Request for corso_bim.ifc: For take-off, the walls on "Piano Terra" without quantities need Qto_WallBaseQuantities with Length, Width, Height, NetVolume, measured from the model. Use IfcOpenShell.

First a look at what the model holds.

```python
import ifcopenshell
import ifcopenshell.util.element
import ifcopenshell.util.unit

model = ifcopenshell.open("corso_bim.ifc")
print(model.schema)
for unit_type in ("LENGTHUNIT", "AREAUNIT", "VOLUMEUNIT"):
    print(unit_type, ifcopenshell.util.unit.calculate_unit_scale(model, unit_type))
storey = next(s for s in model.by_type("IfcBuildingStorey") if s.Name == "Piano Terra")
walls = [e for e in ifcopenshell.util.element.get_decomposition(storey) if e.is_a("IfcWall")]
for e in sorted(walls, key=lambda e: e.id()):
    print(e.id(), e.is_a(), e.Name, list(ifcopenshell.util.element.get_psets(e, qtos_only=True)), sep=" | ")
```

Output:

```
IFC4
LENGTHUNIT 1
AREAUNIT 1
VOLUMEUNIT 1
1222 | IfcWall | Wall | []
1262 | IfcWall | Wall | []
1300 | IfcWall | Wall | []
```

```python
import ifcopenshell
import ifcopenshell.api.pset
import ifcopenshell.geom
import ifcopenshell.util.element
import ifcopenshell.util.shape
import ifcopenshell.util.unit

model = ifcopenshell.open("corso_bim.ifc")
unit_scale = ifcopenshell.util.unit.calculate_unit_scale(model)
volume_scale = ifcopenshell.util.unit.calculate_unit_scale(model, "VOLUMEUNIT")
settings = ifcopenshell.geom.settings()

storey = next(s for s in model.by_type("IfcBuildingStorey") if s.Name == "Piano Terra")
walls = [e for e in ifcopenshell.util.element.get_decomposition(storey) if e.is_a("IfcWall")]

for e in sorted(walls, key=lambda e: e.id()):
    if ifcopenshell.util.element.get_psets(e, qtos_only=True, should_inherit=False):
        continue
    # Geometry comes back in metres, in the element's own axes.
    shape = ifcopenshell.geom.create_shape(settings, e)
    values = {
        "Length": ifcopenshell.util.shape.get_x(shape.geometry) / unit_scale,
        "Width": ifcopenshell.util.shape.get_y(shape.geometry) / unit_scale,
        "Height": ifcopenshell.util.shape.get_z(shape.geometry) / unit_scale,
        "NetVolume": ifcopenshell.util.shape.get_volume(shape.geometry) / volume_scale,
    }
    qto = ifcopenshell.api.pset.add_qto(model, product=e, name="Qto_WallBaseQuantities")
    ifcopenshell.api.pset.edit_qto(model, qto=qto, properties=values)
    print(e.id(), {k: round(v, 3) for k, v in values.items()})

model.write("corso_bim_edited.ifc")
```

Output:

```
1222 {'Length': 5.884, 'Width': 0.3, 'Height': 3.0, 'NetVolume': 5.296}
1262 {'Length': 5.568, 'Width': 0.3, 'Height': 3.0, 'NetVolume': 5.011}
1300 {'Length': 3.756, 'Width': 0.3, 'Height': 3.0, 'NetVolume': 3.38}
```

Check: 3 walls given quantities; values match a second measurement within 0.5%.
